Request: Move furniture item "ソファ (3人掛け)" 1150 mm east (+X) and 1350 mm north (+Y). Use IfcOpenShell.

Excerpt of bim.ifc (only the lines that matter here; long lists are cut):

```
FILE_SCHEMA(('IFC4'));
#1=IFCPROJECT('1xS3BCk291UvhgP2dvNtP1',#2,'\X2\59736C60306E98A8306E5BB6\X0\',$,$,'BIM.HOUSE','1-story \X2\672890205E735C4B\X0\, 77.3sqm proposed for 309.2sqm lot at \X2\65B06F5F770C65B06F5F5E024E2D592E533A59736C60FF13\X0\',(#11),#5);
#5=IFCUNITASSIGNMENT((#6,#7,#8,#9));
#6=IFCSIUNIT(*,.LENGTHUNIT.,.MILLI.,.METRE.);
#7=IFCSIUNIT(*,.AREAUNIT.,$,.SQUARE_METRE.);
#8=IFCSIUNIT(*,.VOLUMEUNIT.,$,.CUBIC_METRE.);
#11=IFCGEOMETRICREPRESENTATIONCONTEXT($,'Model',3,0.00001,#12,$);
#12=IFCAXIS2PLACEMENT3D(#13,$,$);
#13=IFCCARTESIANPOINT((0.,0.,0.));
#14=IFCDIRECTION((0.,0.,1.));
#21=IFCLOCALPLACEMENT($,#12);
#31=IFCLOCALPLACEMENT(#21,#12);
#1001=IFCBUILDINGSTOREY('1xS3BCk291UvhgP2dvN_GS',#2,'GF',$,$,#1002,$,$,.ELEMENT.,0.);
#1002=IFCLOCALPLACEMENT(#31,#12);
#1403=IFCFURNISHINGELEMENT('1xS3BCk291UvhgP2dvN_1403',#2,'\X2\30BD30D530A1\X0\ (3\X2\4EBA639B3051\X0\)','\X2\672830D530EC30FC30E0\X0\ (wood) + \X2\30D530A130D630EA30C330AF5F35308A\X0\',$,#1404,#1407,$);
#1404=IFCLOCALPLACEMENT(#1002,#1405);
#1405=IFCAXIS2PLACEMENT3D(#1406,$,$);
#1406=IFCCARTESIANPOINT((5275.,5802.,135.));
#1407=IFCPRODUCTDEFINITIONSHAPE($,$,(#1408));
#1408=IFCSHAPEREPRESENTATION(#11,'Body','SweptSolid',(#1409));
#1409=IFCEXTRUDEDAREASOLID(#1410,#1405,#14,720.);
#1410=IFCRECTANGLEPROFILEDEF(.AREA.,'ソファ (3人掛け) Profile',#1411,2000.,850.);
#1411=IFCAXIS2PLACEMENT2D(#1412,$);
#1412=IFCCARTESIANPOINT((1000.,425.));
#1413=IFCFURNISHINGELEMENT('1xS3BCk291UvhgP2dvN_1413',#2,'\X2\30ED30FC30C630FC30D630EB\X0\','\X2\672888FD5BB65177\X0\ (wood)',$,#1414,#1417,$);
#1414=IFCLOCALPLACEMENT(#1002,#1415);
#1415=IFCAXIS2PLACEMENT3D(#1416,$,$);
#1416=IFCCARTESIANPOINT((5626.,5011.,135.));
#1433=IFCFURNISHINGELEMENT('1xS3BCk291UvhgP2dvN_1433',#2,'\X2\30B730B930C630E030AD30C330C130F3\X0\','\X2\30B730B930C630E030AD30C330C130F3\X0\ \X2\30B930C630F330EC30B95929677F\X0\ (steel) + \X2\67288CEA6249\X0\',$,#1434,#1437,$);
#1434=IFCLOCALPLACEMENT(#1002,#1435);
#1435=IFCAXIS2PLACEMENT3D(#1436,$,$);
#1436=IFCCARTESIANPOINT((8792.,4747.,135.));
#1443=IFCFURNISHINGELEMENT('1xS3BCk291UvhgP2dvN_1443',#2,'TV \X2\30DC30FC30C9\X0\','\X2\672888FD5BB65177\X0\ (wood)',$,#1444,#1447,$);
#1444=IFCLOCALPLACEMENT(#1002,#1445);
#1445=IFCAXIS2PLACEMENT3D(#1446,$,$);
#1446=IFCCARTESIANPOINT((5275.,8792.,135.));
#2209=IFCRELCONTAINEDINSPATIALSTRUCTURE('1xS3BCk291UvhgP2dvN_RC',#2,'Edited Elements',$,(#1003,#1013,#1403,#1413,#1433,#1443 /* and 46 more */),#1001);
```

```python
import ifcopenshell
import ifcopenshell.api.geometry
import ifcopenshell.util.placement

model = ifcopenshell.open("bim.ifc")

item = model.by_guid("1xS3BCk291UvhgP2dvN_1403")
matrix = ifcopenshell.util.placement.get_local_placement(item.ObjectPlacement)
matrix[0, 3] += 1150.0
matrix[1, 3] += 1350.0
ifcopenshell.api.geometry.edit_object_placement(model, product=item, matrix=matrix, is_si=False)

print(ifcopenshell.util.placement.get_local_placement(item.ObjectPlacement).round(3) + 0.0)

model.write("bim_v2.ifc")
```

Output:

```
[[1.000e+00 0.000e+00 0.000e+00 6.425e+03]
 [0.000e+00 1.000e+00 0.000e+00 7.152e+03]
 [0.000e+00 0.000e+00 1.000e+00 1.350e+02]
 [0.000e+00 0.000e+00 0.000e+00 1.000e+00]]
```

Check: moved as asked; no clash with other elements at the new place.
